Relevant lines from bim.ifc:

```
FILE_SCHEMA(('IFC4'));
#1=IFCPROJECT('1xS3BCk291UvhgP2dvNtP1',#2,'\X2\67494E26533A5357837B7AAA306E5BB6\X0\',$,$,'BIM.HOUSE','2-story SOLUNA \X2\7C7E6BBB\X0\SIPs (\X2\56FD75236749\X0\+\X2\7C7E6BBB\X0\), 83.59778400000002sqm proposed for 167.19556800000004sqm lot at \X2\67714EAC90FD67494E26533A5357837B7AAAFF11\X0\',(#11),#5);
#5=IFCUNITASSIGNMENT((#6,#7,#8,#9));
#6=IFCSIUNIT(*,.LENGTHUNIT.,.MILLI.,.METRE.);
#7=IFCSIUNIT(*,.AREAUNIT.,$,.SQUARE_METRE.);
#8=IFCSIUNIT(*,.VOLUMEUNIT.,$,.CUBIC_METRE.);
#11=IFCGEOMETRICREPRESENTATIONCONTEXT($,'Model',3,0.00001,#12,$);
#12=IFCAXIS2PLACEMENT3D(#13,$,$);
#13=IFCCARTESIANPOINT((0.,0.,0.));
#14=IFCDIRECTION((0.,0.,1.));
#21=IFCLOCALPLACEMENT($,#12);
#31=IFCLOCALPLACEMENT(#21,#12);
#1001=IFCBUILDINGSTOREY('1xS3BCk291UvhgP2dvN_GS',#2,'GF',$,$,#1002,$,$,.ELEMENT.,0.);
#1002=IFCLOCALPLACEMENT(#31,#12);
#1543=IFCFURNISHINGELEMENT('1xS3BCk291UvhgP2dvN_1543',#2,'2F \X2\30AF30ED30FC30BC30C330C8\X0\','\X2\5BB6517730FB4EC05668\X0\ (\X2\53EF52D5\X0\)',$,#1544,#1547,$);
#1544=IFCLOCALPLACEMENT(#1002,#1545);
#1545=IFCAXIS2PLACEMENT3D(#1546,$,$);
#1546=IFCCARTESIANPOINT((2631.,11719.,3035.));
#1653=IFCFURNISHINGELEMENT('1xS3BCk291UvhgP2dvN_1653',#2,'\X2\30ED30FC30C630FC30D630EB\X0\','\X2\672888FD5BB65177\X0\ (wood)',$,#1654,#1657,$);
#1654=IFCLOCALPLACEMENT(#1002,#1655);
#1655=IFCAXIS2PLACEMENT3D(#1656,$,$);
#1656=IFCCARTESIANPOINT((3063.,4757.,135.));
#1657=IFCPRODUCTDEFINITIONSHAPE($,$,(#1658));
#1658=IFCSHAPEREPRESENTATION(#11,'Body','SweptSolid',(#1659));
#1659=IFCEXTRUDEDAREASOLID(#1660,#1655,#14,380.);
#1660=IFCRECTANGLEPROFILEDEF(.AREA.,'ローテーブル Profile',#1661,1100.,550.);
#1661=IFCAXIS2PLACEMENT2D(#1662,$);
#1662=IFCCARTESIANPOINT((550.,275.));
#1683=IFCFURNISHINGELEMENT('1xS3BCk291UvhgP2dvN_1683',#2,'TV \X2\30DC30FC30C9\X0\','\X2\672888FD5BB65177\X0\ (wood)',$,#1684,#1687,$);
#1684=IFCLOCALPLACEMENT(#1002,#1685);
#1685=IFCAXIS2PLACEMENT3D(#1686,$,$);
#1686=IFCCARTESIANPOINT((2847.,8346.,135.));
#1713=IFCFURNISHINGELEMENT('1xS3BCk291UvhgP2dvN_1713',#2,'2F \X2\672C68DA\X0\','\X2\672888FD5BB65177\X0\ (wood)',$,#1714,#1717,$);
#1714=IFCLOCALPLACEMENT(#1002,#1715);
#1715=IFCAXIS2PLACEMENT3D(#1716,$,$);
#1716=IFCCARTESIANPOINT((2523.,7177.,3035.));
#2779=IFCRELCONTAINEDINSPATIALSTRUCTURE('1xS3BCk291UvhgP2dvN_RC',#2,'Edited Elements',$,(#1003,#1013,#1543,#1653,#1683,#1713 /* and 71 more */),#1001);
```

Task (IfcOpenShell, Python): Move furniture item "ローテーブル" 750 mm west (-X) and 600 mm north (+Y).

```python
import ifcopenshell
import ifcopenshell.api.geometry
import ifcopenshell.util.placement
import ifcopenshell.util.unit

model = ifcopenshell.open("bim.ifc")
unit_scale = ifcopenshell.util.unit.calculate_unit_scale(model)

item = model.by_id(1653)
matrix = ifcopenshell.util.placement.get_local_placement(item.ObjectPlacement)
matrix[0, 3] -= 0.75 / unit_scale
matrix[1, 3] += 0.6 / unit_scale
ifcopenshell.api.geometry.edit_object_placement(model, product=item, matrix=matrix, is_si=False)

print(ifcopenshell.util.placement.get_local_placement(item.ObjectPlacement).round(3) + 0.0)

model.write("bim_edited.ifc")
```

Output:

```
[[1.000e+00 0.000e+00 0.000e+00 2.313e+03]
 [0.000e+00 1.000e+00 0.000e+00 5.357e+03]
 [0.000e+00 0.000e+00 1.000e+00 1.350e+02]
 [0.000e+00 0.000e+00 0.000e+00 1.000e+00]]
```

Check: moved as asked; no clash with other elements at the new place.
